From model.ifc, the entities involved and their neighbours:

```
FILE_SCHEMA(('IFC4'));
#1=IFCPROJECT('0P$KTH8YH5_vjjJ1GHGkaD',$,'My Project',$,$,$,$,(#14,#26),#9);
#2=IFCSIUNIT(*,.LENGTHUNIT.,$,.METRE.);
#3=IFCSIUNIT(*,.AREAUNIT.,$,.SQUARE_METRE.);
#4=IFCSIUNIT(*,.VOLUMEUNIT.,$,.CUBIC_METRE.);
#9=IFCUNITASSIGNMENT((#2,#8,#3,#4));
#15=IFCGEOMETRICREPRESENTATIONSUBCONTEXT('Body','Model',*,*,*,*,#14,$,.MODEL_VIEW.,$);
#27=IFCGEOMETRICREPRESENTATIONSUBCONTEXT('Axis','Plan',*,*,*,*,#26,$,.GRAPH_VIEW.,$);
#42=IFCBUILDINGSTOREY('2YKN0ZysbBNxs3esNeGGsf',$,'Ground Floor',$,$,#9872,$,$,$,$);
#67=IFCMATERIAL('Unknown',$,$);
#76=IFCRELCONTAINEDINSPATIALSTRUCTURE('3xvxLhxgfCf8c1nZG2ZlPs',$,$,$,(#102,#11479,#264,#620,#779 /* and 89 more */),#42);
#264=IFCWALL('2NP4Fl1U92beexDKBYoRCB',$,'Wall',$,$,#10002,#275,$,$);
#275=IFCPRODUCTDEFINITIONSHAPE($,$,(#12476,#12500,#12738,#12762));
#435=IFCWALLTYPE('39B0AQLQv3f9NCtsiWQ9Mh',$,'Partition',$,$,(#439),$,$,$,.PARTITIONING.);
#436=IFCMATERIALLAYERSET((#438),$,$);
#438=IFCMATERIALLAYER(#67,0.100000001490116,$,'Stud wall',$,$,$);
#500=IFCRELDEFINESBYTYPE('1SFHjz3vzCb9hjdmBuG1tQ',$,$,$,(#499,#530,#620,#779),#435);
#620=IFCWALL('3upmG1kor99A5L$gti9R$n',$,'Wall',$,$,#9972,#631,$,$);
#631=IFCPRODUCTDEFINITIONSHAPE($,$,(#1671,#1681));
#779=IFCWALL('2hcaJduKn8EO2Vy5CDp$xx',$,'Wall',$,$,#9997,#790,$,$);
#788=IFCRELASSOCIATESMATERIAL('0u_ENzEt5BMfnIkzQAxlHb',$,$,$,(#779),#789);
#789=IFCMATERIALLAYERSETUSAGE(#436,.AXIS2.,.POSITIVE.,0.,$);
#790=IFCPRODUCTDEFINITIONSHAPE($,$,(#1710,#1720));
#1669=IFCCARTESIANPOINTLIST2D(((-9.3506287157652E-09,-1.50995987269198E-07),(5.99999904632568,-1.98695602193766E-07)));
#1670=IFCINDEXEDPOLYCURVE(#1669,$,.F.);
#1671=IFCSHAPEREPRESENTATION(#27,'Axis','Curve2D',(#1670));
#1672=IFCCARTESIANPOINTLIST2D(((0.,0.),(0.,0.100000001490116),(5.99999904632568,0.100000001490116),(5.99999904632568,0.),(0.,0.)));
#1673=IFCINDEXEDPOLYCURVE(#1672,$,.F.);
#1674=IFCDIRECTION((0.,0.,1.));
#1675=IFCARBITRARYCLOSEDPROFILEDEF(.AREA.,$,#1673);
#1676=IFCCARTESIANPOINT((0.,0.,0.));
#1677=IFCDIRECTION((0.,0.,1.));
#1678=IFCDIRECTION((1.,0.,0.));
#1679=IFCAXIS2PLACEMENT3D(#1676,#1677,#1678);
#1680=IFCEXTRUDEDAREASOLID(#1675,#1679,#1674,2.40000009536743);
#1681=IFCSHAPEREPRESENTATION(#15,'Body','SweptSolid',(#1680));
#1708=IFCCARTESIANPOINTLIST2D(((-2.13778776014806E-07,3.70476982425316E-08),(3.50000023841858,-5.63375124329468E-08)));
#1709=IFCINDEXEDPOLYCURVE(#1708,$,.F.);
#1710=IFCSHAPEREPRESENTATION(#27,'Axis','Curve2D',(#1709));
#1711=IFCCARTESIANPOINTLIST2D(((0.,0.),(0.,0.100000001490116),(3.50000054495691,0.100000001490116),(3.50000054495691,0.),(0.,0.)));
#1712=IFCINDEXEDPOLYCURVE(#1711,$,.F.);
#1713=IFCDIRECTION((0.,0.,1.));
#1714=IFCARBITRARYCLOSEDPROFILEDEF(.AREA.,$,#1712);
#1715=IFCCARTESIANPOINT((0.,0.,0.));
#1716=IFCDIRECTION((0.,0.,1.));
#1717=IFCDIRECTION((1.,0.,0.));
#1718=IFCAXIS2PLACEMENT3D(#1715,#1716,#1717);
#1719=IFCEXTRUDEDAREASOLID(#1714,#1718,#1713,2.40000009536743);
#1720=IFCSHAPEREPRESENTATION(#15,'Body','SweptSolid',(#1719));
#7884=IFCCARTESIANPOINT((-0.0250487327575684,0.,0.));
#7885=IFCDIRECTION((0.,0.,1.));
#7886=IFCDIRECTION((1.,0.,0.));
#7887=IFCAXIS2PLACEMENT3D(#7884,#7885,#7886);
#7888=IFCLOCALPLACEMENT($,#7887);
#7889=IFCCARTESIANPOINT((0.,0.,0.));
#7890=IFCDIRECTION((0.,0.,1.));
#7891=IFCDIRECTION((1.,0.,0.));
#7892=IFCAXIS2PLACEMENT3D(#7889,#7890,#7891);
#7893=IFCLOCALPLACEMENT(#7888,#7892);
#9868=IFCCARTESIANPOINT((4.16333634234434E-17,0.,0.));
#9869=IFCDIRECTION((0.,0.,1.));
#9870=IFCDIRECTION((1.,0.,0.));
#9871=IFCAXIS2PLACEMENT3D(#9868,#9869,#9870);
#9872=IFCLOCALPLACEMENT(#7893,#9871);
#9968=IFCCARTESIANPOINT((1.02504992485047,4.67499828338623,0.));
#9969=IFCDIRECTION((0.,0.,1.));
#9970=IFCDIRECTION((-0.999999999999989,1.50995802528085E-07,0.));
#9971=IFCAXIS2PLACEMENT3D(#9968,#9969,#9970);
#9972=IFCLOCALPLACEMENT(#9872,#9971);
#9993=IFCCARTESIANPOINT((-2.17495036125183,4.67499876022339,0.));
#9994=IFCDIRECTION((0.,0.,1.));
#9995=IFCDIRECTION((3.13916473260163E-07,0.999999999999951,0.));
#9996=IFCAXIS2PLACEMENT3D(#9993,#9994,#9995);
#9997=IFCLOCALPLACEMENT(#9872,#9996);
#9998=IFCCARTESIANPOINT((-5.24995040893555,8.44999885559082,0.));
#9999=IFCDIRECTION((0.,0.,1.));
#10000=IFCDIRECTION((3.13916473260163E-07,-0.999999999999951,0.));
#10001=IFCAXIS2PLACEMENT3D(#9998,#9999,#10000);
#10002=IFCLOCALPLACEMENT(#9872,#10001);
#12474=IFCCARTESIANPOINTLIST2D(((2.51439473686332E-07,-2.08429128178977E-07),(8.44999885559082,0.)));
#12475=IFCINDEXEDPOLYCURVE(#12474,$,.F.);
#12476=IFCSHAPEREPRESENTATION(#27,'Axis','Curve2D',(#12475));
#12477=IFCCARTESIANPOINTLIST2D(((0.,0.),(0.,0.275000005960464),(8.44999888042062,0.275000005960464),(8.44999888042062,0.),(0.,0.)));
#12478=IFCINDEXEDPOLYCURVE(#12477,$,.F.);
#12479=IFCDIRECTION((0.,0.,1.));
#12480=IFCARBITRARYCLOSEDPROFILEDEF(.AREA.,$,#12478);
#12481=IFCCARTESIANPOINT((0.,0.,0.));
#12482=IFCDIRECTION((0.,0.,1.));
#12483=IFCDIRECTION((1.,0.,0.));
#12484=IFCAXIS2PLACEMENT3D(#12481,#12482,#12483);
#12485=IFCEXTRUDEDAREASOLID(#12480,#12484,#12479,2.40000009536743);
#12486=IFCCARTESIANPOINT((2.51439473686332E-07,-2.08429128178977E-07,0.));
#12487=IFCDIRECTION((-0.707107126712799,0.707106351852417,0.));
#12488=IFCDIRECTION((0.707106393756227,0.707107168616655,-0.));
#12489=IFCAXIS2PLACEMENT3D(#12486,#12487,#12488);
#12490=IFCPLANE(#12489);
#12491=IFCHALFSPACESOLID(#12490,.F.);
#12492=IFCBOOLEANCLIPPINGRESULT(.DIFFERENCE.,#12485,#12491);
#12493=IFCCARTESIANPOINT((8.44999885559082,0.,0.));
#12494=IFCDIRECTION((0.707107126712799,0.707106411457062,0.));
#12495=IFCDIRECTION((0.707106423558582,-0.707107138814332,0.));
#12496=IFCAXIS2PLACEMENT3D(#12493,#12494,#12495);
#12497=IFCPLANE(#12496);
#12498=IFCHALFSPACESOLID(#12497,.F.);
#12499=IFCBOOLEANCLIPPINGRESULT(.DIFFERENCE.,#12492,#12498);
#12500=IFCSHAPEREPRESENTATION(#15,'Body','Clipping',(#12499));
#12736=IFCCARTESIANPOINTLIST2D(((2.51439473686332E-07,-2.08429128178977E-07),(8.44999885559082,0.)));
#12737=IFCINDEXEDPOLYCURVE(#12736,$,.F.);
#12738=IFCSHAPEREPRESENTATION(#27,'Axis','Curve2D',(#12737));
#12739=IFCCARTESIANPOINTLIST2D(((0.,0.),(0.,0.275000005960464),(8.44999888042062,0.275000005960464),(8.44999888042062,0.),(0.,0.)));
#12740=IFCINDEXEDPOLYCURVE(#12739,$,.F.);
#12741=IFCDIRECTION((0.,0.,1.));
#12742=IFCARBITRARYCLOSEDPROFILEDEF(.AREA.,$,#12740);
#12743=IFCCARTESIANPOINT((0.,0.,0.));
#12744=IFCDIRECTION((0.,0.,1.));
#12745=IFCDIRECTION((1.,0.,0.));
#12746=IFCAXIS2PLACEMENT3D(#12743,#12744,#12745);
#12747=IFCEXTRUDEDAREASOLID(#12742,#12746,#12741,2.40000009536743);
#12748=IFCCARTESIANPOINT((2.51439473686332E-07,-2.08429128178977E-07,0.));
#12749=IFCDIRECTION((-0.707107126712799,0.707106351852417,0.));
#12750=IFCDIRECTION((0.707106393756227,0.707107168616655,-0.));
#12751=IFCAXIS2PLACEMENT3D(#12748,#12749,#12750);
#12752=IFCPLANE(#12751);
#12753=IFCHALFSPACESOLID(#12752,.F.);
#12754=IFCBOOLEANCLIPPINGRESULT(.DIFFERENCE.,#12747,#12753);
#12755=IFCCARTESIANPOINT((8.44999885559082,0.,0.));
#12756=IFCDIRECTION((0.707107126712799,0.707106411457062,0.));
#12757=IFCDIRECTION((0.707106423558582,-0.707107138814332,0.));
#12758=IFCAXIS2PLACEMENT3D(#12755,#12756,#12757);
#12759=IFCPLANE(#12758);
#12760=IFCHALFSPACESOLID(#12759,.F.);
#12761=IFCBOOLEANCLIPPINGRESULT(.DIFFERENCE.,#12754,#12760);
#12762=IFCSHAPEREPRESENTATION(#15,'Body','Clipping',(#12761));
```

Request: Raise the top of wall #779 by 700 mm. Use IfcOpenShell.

```python
import ifcopenshell
import ifcopenshell.geom
import ifcopenshell.util.representation
import ifcopenshell.util.shape
import ifcopenshell.util.unit

model = ifcopenshell.open("model.ifc")
unit_scale = ifcopenshell.util.unit.calculate_unit_scale(model)
settings = ifcopenshell.geom.settings()


def volume(element):
    """Net volume in cubic metres, openings subtracted."""
    shape = ifcopenshell.geom.create_shape(settings, element)
    return ifcopenshell.util.shape.get_volume(shape.geometry)


wall = model.by_id(779)
before = volume(wall)

body = ifcopenshell.util.representation.get_representation(wall, "Model", "Body")
solid = body.Items[0]
old_height = solid.Depth
solid.Depth += 0.7 / unit_scale
after = volume(wall)

print(f"height {old_height:g} -> {solid.Depth:g}, volume {before:.3f} -> {after:.3f} m3")

model.write("model-out.ifc")
```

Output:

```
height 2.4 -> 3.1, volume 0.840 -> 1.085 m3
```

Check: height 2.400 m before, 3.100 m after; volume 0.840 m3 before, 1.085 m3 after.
